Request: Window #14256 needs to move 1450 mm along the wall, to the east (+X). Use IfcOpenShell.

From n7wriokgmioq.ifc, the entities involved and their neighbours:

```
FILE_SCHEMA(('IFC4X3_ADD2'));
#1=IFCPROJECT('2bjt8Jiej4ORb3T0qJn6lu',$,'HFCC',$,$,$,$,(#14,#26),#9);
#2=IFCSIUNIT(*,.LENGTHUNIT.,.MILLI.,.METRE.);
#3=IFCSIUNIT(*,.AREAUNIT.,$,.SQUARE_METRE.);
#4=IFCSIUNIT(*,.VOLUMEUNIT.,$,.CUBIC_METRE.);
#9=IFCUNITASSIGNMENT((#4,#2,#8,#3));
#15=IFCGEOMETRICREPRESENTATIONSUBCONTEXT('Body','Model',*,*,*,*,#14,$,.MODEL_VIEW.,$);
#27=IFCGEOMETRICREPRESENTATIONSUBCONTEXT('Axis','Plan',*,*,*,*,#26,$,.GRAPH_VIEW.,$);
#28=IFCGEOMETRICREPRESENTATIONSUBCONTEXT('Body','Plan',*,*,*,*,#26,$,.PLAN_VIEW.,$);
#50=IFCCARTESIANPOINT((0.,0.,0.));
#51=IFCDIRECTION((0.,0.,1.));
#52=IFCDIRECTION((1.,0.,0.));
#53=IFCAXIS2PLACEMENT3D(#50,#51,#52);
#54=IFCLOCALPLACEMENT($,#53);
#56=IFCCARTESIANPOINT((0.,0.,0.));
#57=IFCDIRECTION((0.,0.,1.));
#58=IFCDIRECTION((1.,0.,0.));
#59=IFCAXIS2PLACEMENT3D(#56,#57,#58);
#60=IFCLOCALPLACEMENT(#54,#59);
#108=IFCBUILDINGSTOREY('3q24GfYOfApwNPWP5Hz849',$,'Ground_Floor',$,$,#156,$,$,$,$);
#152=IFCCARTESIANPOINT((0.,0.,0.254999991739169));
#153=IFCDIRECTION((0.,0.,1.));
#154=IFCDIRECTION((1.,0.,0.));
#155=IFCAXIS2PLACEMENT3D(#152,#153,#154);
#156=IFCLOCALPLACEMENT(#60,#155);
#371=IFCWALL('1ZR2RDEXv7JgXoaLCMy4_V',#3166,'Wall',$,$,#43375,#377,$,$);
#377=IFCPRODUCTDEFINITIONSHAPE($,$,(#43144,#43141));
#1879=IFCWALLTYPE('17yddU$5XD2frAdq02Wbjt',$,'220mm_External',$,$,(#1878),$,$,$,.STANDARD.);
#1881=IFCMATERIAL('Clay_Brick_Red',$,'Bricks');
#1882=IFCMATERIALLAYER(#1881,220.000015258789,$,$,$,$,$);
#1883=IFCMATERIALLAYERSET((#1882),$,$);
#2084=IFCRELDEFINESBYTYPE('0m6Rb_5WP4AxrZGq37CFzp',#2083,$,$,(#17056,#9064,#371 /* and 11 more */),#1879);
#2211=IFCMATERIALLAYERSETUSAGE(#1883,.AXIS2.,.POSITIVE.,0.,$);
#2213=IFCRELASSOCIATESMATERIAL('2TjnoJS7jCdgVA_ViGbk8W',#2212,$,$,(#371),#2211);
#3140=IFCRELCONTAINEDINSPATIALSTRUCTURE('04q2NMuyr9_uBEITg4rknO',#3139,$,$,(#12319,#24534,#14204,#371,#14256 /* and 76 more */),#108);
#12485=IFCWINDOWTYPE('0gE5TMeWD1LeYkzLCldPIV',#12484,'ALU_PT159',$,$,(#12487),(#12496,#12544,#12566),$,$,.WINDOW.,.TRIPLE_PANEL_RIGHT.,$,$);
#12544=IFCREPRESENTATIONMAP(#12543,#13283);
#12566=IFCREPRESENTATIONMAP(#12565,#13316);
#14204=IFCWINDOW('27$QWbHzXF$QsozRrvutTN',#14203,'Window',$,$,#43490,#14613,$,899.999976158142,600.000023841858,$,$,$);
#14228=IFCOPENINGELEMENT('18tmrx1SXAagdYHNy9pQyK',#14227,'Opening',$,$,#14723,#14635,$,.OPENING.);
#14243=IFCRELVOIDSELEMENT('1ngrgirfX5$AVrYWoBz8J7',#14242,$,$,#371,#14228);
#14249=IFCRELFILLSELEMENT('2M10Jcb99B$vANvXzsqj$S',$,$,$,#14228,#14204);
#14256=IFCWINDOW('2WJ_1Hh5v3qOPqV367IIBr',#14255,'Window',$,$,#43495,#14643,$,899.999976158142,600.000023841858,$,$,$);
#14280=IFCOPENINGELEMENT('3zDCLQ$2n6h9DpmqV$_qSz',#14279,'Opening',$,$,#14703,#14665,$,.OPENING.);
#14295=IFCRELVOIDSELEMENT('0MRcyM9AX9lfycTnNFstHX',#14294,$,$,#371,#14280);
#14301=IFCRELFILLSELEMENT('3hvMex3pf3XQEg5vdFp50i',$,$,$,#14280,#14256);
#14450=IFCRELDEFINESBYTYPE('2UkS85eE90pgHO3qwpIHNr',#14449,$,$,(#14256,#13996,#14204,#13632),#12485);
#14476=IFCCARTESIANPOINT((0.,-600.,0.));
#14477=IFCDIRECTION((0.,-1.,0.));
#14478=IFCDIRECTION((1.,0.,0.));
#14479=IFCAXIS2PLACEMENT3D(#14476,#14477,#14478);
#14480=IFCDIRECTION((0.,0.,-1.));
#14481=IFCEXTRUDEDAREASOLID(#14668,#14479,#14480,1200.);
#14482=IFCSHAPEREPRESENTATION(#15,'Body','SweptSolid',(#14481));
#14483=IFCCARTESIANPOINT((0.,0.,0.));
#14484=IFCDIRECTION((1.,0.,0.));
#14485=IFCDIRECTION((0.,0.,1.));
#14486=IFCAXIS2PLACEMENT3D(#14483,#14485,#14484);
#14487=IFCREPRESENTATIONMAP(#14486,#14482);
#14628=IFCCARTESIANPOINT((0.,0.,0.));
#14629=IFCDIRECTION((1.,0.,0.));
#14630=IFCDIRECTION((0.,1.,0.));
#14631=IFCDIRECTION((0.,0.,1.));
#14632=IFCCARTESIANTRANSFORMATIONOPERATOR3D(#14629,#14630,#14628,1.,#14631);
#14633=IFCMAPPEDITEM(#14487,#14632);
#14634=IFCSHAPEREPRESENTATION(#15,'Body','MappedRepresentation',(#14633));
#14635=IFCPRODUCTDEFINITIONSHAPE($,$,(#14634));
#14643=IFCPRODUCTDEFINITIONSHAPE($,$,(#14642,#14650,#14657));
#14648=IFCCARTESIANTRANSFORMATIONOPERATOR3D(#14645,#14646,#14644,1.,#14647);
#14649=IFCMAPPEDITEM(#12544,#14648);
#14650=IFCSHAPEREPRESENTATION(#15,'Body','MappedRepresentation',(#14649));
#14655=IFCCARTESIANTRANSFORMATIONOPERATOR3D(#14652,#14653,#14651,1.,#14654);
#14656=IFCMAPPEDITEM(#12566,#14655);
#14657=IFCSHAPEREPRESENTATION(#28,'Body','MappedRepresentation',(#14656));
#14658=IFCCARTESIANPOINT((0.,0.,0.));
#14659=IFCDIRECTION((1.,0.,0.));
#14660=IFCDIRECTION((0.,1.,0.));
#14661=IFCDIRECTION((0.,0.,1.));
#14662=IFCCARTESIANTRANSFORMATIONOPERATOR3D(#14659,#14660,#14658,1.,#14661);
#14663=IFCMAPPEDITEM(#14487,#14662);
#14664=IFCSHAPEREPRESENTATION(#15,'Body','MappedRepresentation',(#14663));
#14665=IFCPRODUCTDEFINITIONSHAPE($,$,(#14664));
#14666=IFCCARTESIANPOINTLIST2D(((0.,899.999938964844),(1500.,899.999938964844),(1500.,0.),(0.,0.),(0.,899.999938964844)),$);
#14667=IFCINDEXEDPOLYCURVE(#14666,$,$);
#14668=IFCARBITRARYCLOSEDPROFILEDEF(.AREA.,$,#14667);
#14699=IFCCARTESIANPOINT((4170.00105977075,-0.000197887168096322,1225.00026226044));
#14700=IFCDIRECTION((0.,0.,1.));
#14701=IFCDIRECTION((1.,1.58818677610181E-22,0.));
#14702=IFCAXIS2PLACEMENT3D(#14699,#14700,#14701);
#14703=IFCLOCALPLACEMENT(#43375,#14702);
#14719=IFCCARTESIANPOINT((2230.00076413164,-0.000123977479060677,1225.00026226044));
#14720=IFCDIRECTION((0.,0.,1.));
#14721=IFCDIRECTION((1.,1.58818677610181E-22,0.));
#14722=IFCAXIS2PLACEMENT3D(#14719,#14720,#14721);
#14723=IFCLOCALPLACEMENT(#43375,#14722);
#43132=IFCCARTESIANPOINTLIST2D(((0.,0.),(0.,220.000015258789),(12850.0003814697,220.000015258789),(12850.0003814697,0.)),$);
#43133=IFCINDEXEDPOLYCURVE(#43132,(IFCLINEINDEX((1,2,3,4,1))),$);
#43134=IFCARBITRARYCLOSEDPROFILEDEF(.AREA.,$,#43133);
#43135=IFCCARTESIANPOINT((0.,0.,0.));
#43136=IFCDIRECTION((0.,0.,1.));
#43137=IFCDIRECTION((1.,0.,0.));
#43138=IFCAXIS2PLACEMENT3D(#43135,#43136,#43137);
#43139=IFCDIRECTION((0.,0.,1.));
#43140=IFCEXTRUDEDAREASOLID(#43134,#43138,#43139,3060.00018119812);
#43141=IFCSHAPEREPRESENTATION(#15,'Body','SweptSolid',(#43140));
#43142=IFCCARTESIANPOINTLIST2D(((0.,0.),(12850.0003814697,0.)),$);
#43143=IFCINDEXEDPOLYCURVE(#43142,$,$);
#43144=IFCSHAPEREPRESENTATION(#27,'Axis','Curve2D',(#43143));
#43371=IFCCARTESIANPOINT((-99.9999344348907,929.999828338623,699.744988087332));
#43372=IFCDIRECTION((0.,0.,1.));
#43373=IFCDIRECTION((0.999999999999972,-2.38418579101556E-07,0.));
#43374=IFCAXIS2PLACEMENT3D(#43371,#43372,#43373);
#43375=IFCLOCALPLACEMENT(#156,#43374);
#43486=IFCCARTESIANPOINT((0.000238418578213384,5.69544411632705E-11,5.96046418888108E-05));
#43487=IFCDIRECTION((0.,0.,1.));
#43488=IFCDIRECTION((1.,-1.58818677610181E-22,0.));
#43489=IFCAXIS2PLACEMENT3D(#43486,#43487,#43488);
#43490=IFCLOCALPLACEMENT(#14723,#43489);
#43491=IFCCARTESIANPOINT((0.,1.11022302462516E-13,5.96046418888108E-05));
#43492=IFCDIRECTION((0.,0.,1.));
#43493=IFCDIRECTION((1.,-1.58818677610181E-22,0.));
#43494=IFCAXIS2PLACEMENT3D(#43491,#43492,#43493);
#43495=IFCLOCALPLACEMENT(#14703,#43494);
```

```python
import ifcopenshell
import ifcopenshell.api.geometry
import ifcopenshell.util.placement

model = ifcopenshell.open("n7wriokgmioq.ifc")

window = model.by_guid("2WJ_1Hh5v3qOPqV367IIBr")
opening = window.FillsVoids[0].RelatingOpeningElement
wall = opening.VoidsElements[0].RelatingBuildingElement

wall_matrix = ifcopenshell.util.placement.get_local_placement(wall.ObjectPlacement)
shift = wall_matrix[:3, 0] * 1450.0
before = ifcopenshell.util.placement.get_local_placement(window.ObjectPlacement)[:3, 3].copy()

# The window is placed relative to its opening, so it follows when the opening moves.
matrix = ifcopenshell.util.placement.get_local_placement(opening.ObjectPlacement)
matrix[:3, 3] += shift
ifcopenshell.api.geometry.edit_object_placement(
    model, product=opening, matrix=matrix, is_si=False, should_transform_children=True
)

after = ifcopenshell.util.placement.get_local_placement(window.ObjectPlacement)[:3, 3]
print("window moved by", (after - before).round(3) + 0.0)

model.write("n7wriokgmioq_v2.ifc")
```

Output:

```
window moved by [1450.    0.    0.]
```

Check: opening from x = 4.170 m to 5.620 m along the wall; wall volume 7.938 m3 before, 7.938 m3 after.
